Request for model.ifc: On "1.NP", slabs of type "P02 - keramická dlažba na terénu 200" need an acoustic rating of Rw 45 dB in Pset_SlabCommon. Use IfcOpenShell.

First a look at what the model holds.

```python
import ifcopenshell
import ifcopenshell.util.element

model = ifcopenshell.open("model.ifc")
print(model.schema)
storey = next(s for s in model.by_type("IfcBuildingStorey") if s.Name == "1.NP")
slabs = [e for e in ifcopenshell.util.element.get_decomposition(storey) if e.is_a("IfcSlab")]
seen = {}
for e in slabs:
    element_type = ifcopenshell.util.element.get_type(e)
    key = (element_type.Name if element_type != e and element_type else None, ifcopenshell.util.element.get_pset(e, "Pset_SlabCommon", "AcousticRating"))
    seen[key] = seen.get(key, 0) + 1
for (name, value), count in sorted(seen.items(), key=str):
    print(count, "x", name, "|", value)
```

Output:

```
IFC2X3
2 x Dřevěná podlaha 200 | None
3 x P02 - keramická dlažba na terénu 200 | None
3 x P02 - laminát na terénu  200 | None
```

```python
import ifcopenshell
import ifcopenshell.api.pset
import ifcopenshell.util.element

model = ifcopenshell.open("model.ifc")

storey = next(s for s in model.by_type("IfcBuildingStorey") if s.Name == "1.NP")
slabs = [e for e in ifcopenshell.util.element.get_decomposition(storey) if e.is_a("IfcSlab")]

count = 0
for e in slabs:
    element_type = ifcopenshell.util.element.get_type(e)
    if element_type in (None, e) or element_type.Name != "P02 - keramická dlažba na terénu 200":
        continue
    # add_pset returns the element's existing set when there is one.
    pset = ifcopenshell.api.pset.add_pset(model, product=e, name="Pset_SlabCommon")
    ifcopenshell.api.pset.edit_pset(model, pset=pset, properties={"AcousticRating": "Rw 45 dB"})
    count += 1

print(count, "slabs updated")

model.write("model_v2.ifc")
```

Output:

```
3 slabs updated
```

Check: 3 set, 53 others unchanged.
